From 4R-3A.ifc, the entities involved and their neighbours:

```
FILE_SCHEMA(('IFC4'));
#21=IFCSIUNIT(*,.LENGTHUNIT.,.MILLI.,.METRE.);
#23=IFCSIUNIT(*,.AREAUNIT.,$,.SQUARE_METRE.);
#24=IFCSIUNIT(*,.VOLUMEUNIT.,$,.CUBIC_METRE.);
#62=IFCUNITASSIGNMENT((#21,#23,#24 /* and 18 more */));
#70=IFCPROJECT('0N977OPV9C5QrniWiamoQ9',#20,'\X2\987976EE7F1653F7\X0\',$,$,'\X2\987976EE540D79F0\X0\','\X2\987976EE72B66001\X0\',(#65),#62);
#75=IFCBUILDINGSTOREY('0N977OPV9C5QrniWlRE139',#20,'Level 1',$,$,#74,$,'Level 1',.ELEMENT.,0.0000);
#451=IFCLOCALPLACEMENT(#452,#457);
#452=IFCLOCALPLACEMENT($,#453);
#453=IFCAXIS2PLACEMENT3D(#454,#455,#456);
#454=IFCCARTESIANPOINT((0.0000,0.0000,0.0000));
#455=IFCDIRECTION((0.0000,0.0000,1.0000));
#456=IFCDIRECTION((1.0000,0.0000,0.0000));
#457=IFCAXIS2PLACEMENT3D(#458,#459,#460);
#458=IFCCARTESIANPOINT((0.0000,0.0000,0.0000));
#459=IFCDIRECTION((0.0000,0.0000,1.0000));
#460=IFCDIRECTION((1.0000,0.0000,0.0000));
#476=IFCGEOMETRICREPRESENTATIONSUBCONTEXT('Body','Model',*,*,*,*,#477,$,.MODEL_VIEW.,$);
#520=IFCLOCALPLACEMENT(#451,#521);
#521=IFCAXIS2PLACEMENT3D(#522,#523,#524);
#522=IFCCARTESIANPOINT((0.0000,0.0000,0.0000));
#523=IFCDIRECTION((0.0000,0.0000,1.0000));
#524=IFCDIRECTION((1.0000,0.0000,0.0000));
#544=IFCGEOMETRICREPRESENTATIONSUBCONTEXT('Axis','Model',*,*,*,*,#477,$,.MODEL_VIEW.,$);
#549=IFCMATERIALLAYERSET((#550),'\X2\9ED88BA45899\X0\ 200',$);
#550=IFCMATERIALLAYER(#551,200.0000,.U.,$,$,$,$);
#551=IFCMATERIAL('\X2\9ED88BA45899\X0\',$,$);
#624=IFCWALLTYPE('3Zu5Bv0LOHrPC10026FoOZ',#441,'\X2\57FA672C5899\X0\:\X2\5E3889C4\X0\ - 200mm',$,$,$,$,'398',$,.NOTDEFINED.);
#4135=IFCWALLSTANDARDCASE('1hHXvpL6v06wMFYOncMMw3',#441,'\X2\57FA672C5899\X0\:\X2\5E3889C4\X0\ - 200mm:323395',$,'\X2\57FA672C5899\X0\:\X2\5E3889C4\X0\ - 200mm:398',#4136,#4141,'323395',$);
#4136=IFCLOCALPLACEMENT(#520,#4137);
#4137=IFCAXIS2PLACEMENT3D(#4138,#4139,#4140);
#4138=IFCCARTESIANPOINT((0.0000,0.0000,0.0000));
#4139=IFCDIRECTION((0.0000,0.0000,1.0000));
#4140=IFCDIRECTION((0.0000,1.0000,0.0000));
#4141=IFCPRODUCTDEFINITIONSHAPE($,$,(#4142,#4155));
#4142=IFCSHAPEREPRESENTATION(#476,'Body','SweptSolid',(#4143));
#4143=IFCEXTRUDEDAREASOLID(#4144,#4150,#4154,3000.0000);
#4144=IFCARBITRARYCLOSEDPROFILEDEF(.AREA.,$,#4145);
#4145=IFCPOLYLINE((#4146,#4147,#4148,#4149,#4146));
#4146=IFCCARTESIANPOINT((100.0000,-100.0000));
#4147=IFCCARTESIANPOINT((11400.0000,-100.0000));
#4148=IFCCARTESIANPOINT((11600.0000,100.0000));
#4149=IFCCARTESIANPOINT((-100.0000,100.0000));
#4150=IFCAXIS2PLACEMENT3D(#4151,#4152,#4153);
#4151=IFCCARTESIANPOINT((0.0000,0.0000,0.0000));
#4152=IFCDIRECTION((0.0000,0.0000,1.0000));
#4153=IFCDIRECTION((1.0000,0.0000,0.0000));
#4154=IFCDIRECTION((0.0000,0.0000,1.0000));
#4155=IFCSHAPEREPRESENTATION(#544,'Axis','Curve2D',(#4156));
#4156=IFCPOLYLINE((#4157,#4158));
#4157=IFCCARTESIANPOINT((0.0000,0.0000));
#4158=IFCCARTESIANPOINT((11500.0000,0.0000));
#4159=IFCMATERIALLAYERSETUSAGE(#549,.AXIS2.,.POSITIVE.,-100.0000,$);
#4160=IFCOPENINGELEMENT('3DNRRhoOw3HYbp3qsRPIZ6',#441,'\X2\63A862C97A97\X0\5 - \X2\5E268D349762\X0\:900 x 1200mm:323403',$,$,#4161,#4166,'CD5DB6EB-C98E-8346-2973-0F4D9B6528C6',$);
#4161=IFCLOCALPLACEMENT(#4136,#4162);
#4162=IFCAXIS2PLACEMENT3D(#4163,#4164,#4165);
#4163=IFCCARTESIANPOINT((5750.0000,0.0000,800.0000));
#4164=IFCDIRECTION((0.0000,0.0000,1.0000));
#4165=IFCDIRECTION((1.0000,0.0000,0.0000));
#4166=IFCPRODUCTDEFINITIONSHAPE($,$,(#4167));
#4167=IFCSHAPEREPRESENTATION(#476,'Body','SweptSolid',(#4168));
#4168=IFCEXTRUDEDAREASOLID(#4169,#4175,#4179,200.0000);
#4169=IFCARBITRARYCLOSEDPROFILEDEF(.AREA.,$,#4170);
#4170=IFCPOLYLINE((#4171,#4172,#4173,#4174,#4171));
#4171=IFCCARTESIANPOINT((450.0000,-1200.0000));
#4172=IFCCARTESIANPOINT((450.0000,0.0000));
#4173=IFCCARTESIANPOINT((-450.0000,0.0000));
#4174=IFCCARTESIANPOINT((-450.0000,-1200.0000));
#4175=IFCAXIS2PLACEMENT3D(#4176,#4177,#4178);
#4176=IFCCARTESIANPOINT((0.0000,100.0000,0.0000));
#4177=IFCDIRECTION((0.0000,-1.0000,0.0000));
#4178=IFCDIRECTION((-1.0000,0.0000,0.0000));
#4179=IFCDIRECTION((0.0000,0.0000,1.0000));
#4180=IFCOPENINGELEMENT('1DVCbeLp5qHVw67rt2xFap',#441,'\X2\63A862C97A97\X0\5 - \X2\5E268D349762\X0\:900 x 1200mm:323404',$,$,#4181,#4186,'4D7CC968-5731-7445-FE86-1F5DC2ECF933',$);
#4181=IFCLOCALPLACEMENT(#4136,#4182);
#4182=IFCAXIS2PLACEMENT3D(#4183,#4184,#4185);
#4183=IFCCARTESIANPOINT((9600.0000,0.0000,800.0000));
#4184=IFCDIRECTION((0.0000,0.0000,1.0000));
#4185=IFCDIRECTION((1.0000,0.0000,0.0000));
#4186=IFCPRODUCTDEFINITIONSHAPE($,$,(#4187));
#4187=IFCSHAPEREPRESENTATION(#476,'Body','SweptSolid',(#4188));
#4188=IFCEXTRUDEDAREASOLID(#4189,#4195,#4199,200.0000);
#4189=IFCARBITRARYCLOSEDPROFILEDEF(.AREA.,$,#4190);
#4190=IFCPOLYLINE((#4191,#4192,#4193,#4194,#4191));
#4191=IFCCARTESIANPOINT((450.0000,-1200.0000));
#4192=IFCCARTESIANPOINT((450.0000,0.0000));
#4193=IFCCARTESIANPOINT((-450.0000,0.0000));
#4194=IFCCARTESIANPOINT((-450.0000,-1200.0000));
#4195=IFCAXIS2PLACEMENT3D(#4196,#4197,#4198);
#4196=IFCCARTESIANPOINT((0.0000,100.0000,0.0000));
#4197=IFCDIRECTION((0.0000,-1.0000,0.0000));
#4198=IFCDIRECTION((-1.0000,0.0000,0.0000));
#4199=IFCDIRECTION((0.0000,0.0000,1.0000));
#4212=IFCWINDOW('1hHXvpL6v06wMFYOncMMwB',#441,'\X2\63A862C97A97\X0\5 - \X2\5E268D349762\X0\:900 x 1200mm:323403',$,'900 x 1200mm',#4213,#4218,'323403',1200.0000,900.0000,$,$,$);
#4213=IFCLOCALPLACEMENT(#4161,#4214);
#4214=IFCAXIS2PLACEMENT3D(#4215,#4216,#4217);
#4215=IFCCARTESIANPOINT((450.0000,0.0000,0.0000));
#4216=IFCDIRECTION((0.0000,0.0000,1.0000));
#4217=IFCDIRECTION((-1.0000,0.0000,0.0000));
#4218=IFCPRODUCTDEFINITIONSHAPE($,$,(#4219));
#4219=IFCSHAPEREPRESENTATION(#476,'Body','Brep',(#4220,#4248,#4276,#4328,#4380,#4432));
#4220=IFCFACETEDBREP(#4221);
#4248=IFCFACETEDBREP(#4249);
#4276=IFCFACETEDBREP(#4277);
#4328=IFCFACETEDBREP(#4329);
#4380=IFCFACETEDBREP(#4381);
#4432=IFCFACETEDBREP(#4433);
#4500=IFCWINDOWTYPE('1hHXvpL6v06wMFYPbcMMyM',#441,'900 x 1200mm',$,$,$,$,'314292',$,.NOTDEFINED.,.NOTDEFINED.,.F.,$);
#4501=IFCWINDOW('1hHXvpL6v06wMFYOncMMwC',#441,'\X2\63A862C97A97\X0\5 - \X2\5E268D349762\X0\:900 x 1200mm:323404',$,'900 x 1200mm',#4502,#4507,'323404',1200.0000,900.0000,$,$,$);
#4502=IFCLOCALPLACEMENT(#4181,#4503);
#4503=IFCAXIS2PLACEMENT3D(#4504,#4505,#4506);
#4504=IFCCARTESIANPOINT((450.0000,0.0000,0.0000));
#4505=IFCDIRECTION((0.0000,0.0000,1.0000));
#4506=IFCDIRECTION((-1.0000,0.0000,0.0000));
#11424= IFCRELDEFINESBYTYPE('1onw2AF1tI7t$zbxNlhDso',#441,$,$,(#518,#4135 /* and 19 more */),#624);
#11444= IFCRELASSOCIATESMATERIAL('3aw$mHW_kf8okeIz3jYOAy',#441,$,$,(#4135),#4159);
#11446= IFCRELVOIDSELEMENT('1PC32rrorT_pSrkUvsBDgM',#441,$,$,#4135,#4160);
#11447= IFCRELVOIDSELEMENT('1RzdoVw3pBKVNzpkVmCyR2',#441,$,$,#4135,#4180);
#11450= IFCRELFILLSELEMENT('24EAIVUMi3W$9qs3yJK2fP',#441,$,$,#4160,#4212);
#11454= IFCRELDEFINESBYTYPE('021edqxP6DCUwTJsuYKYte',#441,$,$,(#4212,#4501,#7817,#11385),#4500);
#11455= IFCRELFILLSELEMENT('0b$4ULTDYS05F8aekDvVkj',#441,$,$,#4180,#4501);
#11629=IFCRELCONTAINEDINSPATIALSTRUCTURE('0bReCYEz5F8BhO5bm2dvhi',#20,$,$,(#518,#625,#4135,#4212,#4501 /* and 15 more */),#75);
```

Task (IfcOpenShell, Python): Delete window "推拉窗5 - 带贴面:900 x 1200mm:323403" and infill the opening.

```python
import ifcopenshell
import ifcopenshell.api.feature
import ifcopenshell.api.root
import ifcopenshell.geom
import ifcopenshell.util.shape

model = ifcopenshell.open("4R-3A.ifc")
settings = ifcopenshell.geom.settings()


def volume(element):
    """Net volume in cubic metres, openings subtracted."""
    shape = ifcopenshell.geom.create_shape(settings, element)
    return ifcopenshell.util.shape.get_volume(shape.geometry)


window = model.by_id(4212)
opening = window.FillsVoids[0].RelatingOpeningElement
wall = opening.VoidsElements[0].RelatingBuildingElement
before = volume(wall)

ifcopenshell.api.root.remove_product(model, product=window)
ifcopenshell.api.feature.remove_feature(model, feature=opening)

after = volume(wall)

print(f"wall volume {before:.3f} -> {after:.3f} m3")

model.write("4R-3A_edited.ifc")
```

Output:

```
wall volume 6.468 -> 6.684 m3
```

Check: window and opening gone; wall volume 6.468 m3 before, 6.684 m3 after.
